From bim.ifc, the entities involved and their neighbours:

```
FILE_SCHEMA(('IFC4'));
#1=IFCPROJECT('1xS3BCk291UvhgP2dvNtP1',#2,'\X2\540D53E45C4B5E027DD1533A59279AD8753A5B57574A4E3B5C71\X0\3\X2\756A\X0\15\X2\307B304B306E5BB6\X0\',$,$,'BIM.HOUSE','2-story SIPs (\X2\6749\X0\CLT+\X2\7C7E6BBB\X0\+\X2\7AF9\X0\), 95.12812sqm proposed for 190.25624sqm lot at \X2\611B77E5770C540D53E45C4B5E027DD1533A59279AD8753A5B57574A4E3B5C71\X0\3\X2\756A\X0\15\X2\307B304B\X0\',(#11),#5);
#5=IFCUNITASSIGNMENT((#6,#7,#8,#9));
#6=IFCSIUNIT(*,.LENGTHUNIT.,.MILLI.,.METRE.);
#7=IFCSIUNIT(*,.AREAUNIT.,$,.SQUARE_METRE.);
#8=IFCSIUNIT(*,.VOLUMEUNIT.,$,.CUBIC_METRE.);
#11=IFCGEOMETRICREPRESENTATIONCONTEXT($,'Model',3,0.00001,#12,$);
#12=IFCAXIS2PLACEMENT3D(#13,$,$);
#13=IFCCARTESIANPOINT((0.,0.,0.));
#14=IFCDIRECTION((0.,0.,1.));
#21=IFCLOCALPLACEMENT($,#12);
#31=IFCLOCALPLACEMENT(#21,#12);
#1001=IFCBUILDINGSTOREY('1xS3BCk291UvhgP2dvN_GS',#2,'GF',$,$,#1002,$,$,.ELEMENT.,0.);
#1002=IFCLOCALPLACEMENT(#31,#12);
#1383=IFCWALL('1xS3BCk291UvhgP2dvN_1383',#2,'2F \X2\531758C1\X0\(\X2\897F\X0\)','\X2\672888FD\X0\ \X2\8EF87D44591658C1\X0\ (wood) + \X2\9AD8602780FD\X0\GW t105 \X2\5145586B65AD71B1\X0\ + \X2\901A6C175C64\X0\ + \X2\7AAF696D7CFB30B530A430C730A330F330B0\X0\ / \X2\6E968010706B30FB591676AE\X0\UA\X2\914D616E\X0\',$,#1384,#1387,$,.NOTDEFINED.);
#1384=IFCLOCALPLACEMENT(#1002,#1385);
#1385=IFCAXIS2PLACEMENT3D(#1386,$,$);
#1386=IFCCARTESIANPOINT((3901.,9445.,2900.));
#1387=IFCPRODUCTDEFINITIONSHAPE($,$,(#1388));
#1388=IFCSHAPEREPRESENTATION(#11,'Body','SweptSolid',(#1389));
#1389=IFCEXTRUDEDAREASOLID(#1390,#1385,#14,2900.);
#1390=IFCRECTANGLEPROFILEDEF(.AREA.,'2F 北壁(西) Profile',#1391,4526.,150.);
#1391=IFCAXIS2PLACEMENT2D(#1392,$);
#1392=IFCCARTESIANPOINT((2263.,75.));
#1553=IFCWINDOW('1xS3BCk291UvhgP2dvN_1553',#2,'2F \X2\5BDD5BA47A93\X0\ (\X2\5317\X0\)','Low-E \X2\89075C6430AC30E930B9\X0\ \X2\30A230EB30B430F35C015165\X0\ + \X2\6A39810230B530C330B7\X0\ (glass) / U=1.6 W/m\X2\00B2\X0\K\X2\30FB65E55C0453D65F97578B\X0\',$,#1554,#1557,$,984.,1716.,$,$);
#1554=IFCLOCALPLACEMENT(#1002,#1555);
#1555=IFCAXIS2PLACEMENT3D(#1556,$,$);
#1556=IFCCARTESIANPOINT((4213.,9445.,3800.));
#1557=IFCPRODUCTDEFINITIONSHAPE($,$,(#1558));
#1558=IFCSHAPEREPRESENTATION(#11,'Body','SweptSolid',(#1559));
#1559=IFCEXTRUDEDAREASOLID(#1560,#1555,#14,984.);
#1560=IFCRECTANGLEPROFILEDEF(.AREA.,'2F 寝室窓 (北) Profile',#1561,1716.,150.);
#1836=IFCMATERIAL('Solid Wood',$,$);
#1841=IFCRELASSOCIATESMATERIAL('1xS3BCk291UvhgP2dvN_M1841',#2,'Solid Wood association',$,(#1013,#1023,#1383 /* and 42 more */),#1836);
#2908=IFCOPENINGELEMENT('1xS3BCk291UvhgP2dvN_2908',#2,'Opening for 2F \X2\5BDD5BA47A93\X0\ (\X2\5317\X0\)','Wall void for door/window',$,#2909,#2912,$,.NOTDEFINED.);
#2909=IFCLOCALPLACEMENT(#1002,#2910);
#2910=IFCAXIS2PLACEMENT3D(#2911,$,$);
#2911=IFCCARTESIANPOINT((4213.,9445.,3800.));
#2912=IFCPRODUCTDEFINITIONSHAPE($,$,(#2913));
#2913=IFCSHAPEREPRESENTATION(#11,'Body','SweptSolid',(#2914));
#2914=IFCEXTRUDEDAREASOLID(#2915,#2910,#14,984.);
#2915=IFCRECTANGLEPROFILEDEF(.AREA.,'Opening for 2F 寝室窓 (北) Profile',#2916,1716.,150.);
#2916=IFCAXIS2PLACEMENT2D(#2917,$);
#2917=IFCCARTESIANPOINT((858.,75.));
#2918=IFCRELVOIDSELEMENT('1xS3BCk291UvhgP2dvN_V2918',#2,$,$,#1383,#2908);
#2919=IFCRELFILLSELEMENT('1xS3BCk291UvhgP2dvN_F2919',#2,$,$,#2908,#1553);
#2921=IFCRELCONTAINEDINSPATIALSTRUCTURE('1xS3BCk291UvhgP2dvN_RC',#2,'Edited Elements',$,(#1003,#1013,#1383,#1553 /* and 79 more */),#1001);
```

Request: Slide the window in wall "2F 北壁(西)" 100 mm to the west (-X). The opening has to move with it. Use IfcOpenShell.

```python
import ifcopenshell
import ifcopenshell.api.geometry
import ifcopenshell.util.placement
import ifcopenshell.util.unit

model = ifcopenshell.open("bim.ifc")
unit_scale = ifcopenshell.util.unit.calculate_unit_scale(model)

window = model.by_id(1553)
opening = window.FillsVoids[0].RelatingOpeningElement
wall = opening.VoidsElements[0].RelatingBuildingElement

wall_matrix = ifcopenshell.util.placement.get_local_placement(wall.ObjectPlacement)
shift = wall_matrix[:3, 0] * -0.1 / unit_scale
before = ifcopenshell.util.placement.get_local_placement(window.ObjectPlacement)[:3, 3].copy()

# The window is not placed relative to its opening, so move both.
for product in (opening, window):
    matrix = ifcopenshell.util.placement.get_local_placement(product.ObjectPlacement)
    matrix[:3, 3] += shift
    ifcopenshell.api.geometry.edit_object_placement(model, product=product, matrix=matrix, is_si=False)

after = ifcopenshell.util.placement.get_local_placement(window.ObjectPlacement)[:3, 3]
print("window moved by", (after - before).round(3) + 0.0)

model.write("bim_v2.ifc")
```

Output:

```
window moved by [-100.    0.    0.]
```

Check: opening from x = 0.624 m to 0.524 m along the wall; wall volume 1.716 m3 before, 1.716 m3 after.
